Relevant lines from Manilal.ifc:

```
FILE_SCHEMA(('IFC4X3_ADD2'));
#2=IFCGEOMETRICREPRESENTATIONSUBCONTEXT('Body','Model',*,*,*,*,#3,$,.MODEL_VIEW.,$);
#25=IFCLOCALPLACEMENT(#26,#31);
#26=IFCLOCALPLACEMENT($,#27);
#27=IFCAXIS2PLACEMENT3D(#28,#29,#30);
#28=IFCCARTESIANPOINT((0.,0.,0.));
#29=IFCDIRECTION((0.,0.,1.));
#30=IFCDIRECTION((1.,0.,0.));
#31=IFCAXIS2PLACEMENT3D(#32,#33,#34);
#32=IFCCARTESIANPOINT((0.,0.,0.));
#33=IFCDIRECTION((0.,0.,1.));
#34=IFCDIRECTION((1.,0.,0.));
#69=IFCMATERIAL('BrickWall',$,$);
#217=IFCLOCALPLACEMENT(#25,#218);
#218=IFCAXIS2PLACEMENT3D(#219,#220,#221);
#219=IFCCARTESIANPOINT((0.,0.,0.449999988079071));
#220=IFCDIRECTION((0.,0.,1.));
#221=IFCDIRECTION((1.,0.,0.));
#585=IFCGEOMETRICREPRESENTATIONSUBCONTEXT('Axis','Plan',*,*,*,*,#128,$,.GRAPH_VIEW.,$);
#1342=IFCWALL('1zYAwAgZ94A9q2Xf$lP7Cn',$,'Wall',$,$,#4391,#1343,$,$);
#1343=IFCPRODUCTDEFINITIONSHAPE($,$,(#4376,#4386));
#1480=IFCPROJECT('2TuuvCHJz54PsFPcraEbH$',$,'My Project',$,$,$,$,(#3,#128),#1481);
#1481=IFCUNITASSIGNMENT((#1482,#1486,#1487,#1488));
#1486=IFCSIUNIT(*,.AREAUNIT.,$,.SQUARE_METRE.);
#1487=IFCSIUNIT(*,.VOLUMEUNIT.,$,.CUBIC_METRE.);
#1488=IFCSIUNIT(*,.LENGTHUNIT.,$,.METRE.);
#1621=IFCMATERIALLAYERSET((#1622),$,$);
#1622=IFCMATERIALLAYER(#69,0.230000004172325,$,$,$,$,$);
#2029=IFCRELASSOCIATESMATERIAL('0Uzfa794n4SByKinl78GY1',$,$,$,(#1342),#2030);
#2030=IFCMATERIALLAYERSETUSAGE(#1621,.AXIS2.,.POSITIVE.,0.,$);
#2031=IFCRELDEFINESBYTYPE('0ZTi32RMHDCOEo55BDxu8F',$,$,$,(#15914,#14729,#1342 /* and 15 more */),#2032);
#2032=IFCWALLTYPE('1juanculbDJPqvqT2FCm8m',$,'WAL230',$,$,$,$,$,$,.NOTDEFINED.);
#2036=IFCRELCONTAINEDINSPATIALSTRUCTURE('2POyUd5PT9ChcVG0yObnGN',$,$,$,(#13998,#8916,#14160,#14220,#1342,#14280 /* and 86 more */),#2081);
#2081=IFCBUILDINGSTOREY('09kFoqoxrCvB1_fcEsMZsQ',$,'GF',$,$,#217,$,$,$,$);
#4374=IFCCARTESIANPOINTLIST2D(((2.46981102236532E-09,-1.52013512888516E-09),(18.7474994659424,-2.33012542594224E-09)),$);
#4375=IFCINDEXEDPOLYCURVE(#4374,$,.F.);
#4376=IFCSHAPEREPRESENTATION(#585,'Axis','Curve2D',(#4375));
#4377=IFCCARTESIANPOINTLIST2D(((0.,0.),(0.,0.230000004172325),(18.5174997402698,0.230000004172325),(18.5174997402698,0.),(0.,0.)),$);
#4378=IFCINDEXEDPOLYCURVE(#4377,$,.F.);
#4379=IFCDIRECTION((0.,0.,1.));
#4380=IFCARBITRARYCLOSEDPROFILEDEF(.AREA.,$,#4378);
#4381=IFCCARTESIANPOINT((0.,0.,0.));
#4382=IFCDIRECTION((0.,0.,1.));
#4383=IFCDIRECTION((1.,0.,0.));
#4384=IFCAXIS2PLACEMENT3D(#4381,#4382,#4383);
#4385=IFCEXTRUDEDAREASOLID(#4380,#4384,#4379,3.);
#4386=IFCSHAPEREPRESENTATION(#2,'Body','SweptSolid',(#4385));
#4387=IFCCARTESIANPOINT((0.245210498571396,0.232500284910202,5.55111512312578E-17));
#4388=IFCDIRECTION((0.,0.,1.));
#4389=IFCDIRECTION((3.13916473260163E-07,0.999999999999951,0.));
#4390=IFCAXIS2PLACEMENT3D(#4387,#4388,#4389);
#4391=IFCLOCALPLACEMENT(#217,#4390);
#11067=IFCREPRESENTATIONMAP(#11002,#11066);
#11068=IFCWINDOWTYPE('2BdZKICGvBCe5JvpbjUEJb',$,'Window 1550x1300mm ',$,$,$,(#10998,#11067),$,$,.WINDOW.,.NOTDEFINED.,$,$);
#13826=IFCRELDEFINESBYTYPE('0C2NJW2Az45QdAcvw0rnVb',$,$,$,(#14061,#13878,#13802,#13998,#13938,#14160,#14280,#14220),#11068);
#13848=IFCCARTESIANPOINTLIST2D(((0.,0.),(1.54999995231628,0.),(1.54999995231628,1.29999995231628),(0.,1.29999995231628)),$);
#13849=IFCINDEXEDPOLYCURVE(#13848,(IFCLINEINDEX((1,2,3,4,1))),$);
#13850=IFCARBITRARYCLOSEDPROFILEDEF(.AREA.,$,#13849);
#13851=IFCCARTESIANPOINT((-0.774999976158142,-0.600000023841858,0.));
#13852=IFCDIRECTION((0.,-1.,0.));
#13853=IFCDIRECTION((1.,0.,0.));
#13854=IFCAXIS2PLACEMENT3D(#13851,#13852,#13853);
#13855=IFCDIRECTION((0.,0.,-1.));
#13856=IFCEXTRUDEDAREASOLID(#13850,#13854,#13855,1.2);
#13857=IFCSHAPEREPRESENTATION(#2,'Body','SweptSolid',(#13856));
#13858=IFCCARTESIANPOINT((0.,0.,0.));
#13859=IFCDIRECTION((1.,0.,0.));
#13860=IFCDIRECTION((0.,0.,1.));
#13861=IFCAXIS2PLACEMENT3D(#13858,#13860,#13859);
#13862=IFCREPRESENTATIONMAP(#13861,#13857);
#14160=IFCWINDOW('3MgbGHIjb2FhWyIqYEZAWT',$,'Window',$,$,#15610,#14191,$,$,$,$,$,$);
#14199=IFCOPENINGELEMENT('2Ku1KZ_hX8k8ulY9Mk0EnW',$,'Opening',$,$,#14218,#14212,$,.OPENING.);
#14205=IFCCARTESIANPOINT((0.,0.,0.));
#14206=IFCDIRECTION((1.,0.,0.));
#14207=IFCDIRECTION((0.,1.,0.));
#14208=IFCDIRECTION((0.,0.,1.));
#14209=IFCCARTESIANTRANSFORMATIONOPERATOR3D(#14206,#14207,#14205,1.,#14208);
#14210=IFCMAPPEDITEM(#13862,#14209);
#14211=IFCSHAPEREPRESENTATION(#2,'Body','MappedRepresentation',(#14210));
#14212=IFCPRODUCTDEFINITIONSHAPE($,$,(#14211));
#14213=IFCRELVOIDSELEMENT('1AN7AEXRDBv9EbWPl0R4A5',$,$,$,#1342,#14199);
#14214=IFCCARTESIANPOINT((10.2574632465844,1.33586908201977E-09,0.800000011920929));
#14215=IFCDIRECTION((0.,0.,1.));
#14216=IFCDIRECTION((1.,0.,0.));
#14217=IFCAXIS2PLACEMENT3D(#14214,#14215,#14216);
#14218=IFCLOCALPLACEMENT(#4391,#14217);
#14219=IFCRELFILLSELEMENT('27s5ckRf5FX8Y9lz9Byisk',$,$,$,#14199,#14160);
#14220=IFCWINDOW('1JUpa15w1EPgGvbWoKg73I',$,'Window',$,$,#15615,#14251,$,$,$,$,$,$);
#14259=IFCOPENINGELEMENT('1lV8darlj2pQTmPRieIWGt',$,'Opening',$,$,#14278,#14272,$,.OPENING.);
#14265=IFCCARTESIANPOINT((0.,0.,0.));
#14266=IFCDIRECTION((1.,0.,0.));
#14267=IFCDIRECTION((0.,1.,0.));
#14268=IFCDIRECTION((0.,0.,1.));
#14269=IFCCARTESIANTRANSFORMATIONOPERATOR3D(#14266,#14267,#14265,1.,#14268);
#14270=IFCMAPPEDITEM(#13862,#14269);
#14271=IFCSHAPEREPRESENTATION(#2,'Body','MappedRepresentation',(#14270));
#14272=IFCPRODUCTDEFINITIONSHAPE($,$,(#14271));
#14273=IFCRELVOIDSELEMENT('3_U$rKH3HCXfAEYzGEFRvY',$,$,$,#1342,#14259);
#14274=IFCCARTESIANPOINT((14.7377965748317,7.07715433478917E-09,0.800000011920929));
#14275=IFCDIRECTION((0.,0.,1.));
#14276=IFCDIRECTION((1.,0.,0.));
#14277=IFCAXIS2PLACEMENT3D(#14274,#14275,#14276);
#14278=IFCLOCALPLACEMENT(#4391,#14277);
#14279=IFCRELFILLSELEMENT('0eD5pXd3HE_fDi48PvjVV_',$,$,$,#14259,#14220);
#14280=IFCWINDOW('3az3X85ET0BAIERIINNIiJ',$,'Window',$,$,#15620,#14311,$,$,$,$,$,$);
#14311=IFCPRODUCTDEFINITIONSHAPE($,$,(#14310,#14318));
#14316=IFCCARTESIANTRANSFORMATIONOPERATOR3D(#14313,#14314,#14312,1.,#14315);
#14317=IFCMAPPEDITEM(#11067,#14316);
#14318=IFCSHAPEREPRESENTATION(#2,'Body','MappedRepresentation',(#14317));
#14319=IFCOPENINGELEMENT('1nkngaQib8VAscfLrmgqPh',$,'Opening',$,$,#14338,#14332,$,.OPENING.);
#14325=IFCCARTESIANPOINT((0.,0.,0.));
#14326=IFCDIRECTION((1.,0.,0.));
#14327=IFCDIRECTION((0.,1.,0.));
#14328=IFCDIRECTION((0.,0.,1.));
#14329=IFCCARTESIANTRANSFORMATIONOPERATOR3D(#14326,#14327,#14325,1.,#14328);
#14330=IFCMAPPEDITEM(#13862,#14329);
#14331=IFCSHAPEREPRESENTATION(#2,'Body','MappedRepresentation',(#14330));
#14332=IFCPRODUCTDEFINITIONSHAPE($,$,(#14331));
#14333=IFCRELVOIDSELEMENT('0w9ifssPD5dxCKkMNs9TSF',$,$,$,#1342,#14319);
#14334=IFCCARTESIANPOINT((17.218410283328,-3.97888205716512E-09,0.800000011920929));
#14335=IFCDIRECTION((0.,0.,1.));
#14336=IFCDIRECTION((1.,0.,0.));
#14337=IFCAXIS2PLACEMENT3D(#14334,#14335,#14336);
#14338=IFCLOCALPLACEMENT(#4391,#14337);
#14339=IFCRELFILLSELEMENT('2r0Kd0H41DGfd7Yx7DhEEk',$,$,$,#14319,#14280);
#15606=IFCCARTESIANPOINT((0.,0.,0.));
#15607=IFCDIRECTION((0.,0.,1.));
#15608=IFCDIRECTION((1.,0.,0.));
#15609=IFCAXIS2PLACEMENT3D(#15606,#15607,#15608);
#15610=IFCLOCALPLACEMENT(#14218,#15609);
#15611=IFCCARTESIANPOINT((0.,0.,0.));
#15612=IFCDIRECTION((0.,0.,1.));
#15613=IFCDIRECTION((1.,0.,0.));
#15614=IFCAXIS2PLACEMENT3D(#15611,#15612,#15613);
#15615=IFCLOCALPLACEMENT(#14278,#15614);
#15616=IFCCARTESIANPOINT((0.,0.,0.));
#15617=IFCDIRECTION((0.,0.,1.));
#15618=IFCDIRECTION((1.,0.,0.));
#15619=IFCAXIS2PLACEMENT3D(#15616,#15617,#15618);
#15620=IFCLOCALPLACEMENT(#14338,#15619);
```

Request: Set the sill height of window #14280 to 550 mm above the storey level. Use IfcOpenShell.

```python
import numpy as np
import ifcopenshell
import ifcopenshell.api.geometry
import ifcopenshell.geom
import ifcopenshell.util.element
import ifcopenshell.util.placement
import ifcopenshell.util.shape
import ifcopenshell.util.unit

model = ifcopenshell.open("Manilal.ifc")
unit_scale = ifcopenshell.util.unit.calculate_unit_scale(model)

window = model.by_id(14280)
opening = window.FillsVoids[0].RelatingOpeningElement
storey = ifcopenshell.util.element.get_container(window, ifc_class="IfcBuildingStorey")
level = ifcopenshell.util.placement.get_local_placement(storey.ObjectPlacement)[2, 3]

# The opening's origin need not be at the sill, so measure its lowest point.
shape = ifcopenshell.geom.create_shape(ifcopenshell.geom.settings(), opening)
bottom = ifcopenshell.util.shape.get_shape_bottom_elevation(shape, shape.geometry) / unit_scale
dz = level + 0.55 - bottom

shift = np.array([0.0, 0.0, dz])
# The window is placed relative to its opening, so it follows when the opening moves.
matrix = ifcopenshell.util.placement.get_local_placement(opening.ObjectPlacement)
matrix[:3, 3] += shift
ifcopenshell.api.geometry.edit_object_placement(
    model, product=opening, matrix=matrix, is_si=False, should_transform_children=True
)

print(f"moved by {dz * unit_scale:+.3f} m")

model.write("Manilal_edited.ifc")
```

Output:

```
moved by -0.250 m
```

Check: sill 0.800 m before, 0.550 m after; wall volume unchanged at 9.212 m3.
